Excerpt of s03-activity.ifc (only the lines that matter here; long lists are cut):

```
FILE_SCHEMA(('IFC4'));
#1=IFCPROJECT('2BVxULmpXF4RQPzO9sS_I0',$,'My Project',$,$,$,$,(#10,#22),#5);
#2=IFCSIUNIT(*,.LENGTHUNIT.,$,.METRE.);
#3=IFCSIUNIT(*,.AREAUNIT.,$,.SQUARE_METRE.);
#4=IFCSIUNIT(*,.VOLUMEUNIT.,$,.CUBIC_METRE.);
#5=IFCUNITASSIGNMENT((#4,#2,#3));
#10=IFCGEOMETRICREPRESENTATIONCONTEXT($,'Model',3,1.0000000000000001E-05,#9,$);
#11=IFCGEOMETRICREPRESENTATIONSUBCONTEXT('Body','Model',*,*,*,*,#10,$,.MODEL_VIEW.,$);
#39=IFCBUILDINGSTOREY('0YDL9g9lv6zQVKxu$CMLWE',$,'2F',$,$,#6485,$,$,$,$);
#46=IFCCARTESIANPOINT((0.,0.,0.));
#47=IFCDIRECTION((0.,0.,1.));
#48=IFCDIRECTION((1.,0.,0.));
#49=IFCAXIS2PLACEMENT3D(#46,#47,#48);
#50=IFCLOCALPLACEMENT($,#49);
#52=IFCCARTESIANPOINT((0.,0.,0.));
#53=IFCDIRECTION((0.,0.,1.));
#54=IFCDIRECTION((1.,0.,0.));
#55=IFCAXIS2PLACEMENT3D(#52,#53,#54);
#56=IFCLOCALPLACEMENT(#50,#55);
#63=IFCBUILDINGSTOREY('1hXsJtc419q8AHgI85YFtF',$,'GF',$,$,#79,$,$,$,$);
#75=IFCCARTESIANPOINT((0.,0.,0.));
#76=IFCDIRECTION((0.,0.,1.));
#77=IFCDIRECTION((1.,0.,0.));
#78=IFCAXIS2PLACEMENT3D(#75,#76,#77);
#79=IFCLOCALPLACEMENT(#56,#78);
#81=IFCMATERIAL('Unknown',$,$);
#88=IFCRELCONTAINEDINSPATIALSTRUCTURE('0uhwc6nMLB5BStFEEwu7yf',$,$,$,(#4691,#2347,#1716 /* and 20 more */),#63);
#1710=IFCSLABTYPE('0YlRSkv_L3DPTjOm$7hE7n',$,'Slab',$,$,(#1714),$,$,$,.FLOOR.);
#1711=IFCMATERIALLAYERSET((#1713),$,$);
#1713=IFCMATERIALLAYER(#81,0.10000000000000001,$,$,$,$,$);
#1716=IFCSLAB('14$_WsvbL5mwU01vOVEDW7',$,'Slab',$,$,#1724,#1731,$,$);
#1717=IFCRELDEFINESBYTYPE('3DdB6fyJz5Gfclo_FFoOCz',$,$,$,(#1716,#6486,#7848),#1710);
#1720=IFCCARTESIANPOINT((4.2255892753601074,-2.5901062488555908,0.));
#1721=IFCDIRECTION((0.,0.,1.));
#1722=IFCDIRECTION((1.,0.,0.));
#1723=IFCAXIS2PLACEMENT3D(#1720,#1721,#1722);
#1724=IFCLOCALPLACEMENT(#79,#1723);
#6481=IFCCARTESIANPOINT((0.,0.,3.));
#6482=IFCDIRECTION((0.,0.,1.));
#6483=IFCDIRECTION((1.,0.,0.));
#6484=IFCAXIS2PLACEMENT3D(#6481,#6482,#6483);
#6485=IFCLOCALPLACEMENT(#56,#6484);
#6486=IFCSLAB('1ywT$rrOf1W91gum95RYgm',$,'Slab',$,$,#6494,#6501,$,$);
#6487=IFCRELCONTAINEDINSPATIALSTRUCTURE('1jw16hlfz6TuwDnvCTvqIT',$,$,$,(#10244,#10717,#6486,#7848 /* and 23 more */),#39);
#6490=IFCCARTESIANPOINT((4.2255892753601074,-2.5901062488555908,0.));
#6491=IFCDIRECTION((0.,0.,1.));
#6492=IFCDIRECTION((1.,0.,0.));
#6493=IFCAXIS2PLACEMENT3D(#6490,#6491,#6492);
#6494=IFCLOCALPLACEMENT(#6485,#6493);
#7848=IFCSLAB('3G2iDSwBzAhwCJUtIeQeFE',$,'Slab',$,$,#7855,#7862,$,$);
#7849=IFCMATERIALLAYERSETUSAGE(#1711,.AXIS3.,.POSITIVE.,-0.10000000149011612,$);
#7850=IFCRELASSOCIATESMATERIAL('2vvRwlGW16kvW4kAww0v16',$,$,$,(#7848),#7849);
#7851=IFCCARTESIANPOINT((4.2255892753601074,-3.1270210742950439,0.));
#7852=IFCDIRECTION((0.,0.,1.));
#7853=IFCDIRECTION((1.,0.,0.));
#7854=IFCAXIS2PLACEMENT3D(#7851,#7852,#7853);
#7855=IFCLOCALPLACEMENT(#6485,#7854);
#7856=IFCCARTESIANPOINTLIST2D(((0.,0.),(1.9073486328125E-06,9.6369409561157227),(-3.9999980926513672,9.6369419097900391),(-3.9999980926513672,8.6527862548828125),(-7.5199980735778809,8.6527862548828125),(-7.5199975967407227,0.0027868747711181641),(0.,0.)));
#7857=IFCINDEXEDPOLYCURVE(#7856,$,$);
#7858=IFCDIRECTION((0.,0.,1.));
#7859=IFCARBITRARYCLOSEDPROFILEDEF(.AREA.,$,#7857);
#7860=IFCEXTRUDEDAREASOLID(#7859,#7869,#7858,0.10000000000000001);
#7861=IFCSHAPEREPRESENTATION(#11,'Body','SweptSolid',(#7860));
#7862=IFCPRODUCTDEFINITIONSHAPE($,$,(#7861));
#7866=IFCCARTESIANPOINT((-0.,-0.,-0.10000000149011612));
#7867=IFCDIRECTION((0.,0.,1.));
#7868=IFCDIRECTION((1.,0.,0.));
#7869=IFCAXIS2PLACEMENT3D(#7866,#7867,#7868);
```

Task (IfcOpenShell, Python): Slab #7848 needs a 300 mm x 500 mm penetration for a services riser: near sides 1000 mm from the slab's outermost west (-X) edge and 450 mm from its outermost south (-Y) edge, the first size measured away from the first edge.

```python
import numpy as np
import ifcopenshell
import ifcopenshell.api.feature
import ifcopenshell.api.geometry
import ifcopenshell.api.root
import ifcopenshell.geom
import ifcopenshell.util.placement
import ifcopenshell.util.representation
import ifcopenshell.util.shape
import ifcopenshell.util.unit

model = ifcopenshell.open("s03-activity.ifc")
unit_scale = ifcopenshell.util.unit.calculate_unit_scale(model)
settings = ifcopenshell.geom.settings()


def volume(element):
    """Net volume in cubic metres, openings subtracted."""
    shape = ifcopenshell.geom.create_shape(settings, element)
    return ifcopenshell.util.shape.get_volume(shape.geometry)


slab = model.by_guid("3G2iDSwBzAhwCJUtIeQeFE")
before = volume(slab)

# Extent in the slab's own axes, in metres. The edges named are its -X and -Y sides.
slab_shape = ifcopenshell.geom.create_shape(settings, slab)
vertices = ifcopenshell.util.shape.get_vertices(slab_shape.geometry)
x_min, y_min, bottom = vertices.min(axis=0)
top = vertices[:, 2].max()

opening = ifcopenshell.api.root.create_entity(model, ifc_class="IfcOpeningElement", name="Services riser opening", predefined_type="OPENING")
context = ifcopenshell.util.representation.get_context(model, "Model", "Body", "MODEL_VIEW")
width, depth = 0.3, 0.5
outline = [(0.0, 0.0), (width, 0.0), (width, depth), (0.0, depth), (0.0, 0.0)]
# Overshoot both faces by 50 mm so the cut is clean.
shape = ifcopenshell.api.geometry.add_slab_representation(
    model, context=context, depth=top - bottom + 0.1, polyline=outline
)
ifcopenshell.api.geometry.assign_representation(model, product=opening, representation=shape)

matrix = ifcopenshell.util.placement.get_local_placement(slab.ObjectPlacement)
matrix[:, 3] = matrix @ np.append(np.array([x_min + 1, y_min + 0.45, bottom - 0.05]) / unit_scale, 1.0)
ifcopenshell.api.geometry.edit_object_placement(model, product=opening, matrix=matrix, is_si=False)
ifcopenshell.api.feature.add_feature(model, feature=opening, element=slab)

after = volume(slab)

print(f"slab volume {before:.3f} -> {after:.3f} m3")

model.write("s03-activity_v2.ifc")
```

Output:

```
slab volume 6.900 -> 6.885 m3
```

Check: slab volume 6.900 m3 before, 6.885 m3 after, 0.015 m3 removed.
